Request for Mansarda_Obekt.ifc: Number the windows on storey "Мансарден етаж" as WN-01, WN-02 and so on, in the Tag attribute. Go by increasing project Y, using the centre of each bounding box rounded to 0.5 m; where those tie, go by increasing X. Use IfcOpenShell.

First a look at what the model holds.

```python
import ifcopenshell
import ifcopenshell.util.element
import ifcopenshell.util.placement

model = ifcopenshell.open("Mansarda_Obekt.ifc")
print(model.schema)
storey = next(s for s in model.by_type("IfcBuildingStorey") if s.Name == "Мансарден етаж")
windows = [e for e in ifcopenshell.util.element.get_decomposition(storey) if e.is_a("IfcWindow")]
for e in sorted(windows, key=lambda e: e.id()):
    origin = ifcopenshell.util.placement.get_local_placement(e.ObjectPlacement)[:3, 3]
    print(e.id(), e.Tag, e.Name, origin.round(2) + 0.0, sep=" | ")
```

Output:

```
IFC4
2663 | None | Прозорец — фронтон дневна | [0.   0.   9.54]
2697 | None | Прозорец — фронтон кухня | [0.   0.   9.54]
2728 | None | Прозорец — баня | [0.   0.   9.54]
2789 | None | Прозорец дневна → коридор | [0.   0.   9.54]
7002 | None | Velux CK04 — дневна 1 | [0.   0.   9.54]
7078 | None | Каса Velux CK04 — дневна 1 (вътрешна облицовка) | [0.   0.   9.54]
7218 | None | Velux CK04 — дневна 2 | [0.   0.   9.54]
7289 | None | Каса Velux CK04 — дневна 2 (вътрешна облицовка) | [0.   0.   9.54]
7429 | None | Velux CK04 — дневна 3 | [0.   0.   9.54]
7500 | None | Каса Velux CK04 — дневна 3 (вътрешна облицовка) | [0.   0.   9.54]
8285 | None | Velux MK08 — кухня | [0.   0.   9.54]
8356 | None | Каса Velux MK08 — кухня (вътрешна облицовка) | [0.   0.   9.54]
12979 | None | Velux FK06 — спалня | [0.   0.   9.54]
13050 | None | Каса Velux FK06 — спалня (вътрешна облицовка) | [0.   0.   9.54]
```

```python
import ifcopenshell
import ifcopenshell.geom
import ifcopenshell.util.element
import ifcopenshell.util.shape

model = ifcopenshell.open("Mansarda_Obekt.ifc")
settings = ifcopenshell.geom.settings()
settings.set("use-world-coords", True)


def centre(element):
    shape = ifcopenshell.geom.create_shape(settings, element)
    return ifcopenshell.util.shape.get_bbox_centroid(shape.geometry)


storey = next(s for s in model.by_type("IfcBuildingStorey") if s.Name == "Мансарден етаж")
windows = [e for e in ifcopenshell.util.element.get_decomposition(storey) if e.is_a("IfcWindow")]

# Insertion points can sit at a corner or the storey origin, so sort by the geometry (in metres).
centres = {e: centre(e) for e in windows}
windows.sort(key=lambda e: (round(centres[e][1] / 0.5), centres[e][0]))

for i, e in enumerate(windows, start=1):
    number = f"WN-{i:02d}"
    e.Tag = number
    print(e.id(), number)

model.write("Mansarda_Obekt_edited.ifc")
```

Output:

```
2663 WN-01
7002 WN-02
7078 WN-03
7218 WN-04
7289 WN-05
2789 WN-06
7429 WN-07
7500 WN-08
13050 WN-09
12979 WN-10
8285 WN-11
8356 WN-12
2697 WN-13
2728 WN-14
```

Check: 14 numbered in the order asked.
